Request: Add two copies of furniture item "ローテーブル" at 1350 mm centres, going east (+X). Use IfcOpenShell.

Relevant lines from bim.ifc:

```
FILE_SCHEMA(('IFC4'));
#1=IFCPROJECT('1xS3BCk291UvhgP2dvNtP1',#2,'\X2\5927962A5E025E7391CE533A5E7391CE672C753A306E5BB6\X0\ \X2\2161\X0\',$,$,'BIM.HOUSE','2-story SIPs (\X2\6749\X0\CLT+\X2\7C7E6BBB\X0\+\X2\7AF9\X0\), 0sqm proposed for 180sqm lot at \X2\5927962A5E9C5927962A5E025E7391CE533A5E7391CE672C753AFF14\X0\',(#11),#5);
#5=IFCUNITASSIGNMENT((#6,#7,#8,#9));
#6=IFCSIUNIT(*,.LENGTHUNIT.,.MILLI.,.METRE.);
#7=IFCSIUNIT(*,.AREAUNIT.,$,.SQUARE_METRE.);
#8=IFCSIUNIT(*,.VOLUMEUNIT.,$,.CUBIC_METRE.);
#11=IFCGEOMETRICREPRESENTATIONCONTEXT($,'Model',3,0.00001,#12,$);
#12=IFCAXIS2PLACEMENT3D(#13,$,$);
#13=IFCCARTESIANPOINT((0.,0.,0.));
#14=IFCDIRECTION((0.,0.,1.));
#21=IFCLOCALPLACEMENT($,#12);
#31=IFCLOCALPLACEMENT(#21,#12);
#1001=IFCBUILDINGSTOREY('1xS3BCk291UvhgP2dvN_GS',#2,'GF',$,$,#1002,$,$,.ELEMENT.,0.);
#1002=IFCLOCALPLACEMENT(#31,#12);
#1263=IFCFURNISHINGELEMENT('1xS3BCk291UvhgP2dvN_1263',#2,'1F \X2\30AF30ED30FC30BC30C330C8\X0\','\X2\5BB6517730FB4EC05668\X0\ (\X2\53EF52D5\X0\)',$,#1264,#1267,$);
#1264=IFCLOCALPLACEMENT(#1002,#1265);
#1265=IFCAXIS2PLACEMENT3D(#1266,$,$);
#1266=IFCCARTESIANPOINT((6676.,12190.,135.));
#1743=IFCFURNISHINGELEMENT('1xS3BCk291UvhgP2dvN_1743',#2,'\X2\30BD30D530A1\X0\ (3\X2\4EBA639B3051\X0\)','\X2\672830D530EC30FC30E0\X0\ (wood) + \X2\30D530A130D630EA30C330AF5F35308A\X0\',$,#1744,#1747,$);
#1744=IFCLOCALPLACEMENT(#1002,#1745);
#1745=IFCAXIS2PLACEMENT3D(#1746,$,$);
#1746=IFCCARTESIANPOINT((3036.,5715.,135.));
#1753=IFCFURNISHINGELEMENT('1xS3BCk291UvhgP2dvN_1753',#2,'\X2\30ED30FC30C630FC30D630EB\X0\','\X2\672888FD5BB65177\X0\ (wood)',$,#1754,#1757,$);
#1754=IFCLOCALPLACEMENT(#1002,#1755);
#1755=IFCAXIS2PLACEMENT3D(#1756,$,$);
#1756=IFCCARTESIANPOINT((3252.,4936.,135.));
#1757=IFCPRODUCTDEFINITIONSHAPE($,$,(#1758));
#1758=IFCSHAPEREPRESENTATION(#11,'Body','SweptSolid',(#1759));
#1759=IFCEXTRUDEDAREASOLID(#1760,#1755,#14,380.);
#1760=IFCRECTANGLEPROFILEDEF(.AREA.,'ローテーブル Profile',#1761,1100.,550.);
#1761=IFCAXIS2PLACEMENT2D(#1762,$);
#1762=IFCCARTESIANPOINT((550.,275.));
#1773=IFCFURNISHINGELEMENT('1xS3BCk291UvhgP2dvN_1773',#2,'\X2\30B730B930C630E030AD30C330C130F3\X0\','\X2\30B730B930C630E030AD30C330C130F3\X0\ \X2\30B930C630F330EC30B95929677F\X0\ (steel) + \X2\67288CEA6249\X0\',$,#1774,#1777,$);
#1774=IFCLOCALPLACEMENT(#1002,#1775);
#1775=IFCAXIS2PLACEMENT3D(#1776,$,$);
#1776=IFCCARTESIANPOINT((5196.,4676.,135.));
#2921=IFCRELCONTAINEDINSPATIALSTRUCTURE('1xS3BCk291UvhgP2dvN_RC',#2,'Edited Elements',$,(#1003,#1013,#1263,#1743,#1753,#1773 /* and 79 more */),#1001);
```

```python
import numpy as np
import ifcopenshell
import ifcopenshell.api.geometry
import ifcopenshell.api.root
import ifcopenshell.util.element
import ifcopenshell.util.placement
import ifcopenshell.util.unit

model = ifcopenshell.open("bim.ifc")
unit_scale = ifcopenshell.util.unit.calculate_unit_scale(model)


def reuse_history(source, copy):
    """copy_class also copies each property set's owner history, people and application; keep the originals."""
    for rel in copy.IsDefinedBy:
        if rel.is_a("IfcRelDefinesByProperties") and (history := rel.RelatingPropertyDefinition.OwnerHistory):
            rel.RelatingPropertyDefinition.OwnerHistory = source.OwnerHistory
            ifcopenshell.util.element.remove_deep2(model, history)


source = model.by_id(1753)
base = ifcopenshell.util.placement.get_local_placement(source.ObjectPlacement)
step = np.array([1.0, 0.0, 0.0]) * 1.35 / unit_scale

for i in range(1, 3):
    copy = ifcopenshell.api.root.copy_class(model, product=source)
    copy.Representation = ifcopenshell.util.element.copy_deep(
        model, source.Representation, exclude=["IfcGeometricRepresentationContext", "IfcRepresentationMap"]
    )
    reuse_history(source, copy)
    matrix = base.copy()
    matrix[:3, 3] += i * step
    print("added at", matrix[:3, 3].round(3) + 0.0)
    ifcopenshell.api.geometry.edit_object_placement(model, product=copy, matrix=matrix, is_si=False)

model.write("bim_edited.ifc")
```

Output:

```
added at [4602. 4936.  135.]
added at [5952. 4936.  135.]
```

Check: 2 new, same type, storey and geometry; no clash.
